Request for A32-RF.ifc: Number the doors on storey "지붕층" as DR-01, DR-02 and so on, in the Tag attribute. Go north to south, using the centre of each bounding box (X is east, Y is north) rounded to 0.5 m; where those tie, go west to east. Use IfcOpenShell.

First a look at what the model holds.

```python
import ifcopenshell
import ifcopenshell.util.element
import ifcopenshell.util.placement

model = ifcopenshell.open("A32-RF.ifc")
print(model.schema)
storey = next(s for s in model.by_type("IfcBuildingStorey") if s.Name == "지붕층")
doors = [e for e in ifcopenshell.util.element.get_decomposition(storey) if e.is_a("IfcDoor")]
for e in sorted(doors, key=lambda e: e.id()):
    origin = ifcopenshell.util.placement.get_local_placement(e.ObjectPlacement)[:3, 3]
    print(e.id(), e.Tag, e.Name, origin.round(2) + 0.0, sep=" | ")
```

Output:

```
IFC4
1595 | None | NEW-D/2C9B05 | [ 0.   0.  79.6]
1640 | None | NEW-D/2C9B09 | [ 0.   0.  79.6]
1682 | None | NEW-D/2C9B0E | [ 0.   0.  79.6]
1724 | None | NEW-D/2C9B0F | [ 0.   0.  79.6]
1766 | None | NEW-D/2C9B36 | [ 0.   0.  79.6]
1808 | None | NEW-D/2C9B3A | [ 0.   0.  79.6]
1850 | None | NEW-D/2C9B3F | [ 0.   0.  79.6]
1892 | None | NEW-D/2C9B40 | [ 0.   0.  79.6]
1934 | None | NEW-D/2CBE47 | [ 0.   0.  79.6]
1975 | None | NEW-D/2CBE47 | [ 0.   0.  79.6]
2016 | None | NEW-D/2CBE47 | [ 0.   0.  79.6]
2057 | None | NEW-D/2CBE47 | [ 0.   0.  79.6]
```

```python
import ifcopenshell
import ifcopenshell.geom
import ifcopenshell.util.element
import ifcopenshell.util.shape

model = ifcopenshell.open("A32-RF.ifc")
settings = ifcopenshell.geom.settings()
settings.set("use-world-coords", True)


def centre(element):
    shape = ifcopenshell.geom.create_shape(settings, element)
    return ifcopenshell.util.shape.get_bbox_centroid(shape.geometry)


storey = next(s for s in model.by_type("IfcBuildingStorey") if s.Name == "지붕층")
doors = [e for e in ifcopenshell.util.element.get_decomposition(storey) if e.is_a("IfcDoor")]

# Insertion points can sit at a corner or the storey origin, so sort by the geometry (in metres).
centres = {e: centre(e) for e in doors}
doors.sort(key=lambda e: (-round(centres[e][1] / 0.5), centres[e][0]))

for i, e in enumerate(doors, start=1):
    number = f"DR-{i:02d}"
    e.Tag = number
    print(e.id(), number)

model.write("A32-RF-out.ifc")
```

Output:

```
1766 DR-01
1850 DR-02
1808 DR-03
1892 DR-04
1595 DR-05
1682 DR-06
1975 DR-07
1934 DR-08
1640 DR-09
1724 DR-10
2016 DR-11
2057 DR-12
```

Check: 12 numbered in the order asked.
